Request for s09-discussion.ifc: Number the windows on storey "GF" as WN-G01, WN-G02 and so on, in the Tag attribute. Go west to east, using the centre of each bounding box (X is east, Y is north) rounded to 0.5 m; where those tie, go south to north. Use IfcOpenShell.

First a look at what the model holds.

```python
import ifcopenshell
import ifcopenshell.util.element
import ifcopenshell.util.placement

model = ifcopenshell.open("s09-discussion.ifc")
print(model.schema)
storey = next(s for s in model.by_type("IfcBuildingStorey") if s.Name == "GF")
windows = [e for e in ifcopenshell.util.element.get_decomposition(storey) if e.is_a("IfcWindow")]
for e in sorted(windows, key=lambda e: e.id()):
    origin = ifcopenshell.util.placement.get_local_placement(e.ObjectPlacement)[:3, 3]
    print(e.id(), e.Tag, e.Name, origin.round(2) + 0.0, sep=" | ")
```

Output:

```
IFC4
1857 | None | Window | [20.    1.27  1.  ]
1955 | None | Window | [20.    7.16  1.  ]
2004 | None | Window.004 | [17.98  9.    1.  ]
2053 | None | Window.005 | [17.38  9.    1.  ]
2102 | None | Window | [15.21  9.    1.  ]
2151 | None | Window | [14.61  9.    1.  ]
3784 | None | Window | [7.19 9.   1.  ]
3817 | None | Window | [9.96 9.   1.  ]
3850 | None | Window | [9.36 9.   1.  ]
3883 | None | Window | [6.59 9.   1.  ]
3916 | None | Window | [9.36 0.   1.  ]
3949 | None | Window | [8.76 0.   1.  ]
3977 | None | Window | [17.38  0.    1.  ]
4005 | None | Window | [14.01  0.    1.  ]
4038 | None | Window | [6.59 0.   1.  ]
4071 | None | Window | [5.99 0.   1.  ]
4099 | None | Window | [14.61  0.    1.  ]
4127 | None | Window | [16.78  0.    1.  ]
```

```python
import ifcopenshell
import ifcopenshell.geom
import ifcopenshell.util.element
import ifcopenshell.util.shape

model = ifcopenshell.open("s09-discussion.ifc")
settings = ifcopenshell.geom.settings()
settings.set("use-world-coords", True)


def centre(element):
    shape = ifcopenshell.geom.create_shape(settings, element)
    return ifcopenshell.util.shape.get_bbox_centroid(shape.geometry)


storey = next(s for s in model.by_type("IfcBuildingStorey") if s.Name == "GF")
windows = [e for e in ifcopenshell.util.element.get_decomposition(storey) if e.is_a("IfcWindow")]

# Insertion points can sit at a corner or the storey origin, so sort by the geometry (in metres).
centres = {e: centre(e) for e in windows}
windows.sort(key=lambda e: (round(centres[e][0] / 0.5), centres[e][1]))

for i, e in enumerate(windows, start=1):
    number = f"WN-G{i:02d}"
    e.Tag = number
    print(e.id(), number)

model.write("s09-discussion_updated.ifc")
```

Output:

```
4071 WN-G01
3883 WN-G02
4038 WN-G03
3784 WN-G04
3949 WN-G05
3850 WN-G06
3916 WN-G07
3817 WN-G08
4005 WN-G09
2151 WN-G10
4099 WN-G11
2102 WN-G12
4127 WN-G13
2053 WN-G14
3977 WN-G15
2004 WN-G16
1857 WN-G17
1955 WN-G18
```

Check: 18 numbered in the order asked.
